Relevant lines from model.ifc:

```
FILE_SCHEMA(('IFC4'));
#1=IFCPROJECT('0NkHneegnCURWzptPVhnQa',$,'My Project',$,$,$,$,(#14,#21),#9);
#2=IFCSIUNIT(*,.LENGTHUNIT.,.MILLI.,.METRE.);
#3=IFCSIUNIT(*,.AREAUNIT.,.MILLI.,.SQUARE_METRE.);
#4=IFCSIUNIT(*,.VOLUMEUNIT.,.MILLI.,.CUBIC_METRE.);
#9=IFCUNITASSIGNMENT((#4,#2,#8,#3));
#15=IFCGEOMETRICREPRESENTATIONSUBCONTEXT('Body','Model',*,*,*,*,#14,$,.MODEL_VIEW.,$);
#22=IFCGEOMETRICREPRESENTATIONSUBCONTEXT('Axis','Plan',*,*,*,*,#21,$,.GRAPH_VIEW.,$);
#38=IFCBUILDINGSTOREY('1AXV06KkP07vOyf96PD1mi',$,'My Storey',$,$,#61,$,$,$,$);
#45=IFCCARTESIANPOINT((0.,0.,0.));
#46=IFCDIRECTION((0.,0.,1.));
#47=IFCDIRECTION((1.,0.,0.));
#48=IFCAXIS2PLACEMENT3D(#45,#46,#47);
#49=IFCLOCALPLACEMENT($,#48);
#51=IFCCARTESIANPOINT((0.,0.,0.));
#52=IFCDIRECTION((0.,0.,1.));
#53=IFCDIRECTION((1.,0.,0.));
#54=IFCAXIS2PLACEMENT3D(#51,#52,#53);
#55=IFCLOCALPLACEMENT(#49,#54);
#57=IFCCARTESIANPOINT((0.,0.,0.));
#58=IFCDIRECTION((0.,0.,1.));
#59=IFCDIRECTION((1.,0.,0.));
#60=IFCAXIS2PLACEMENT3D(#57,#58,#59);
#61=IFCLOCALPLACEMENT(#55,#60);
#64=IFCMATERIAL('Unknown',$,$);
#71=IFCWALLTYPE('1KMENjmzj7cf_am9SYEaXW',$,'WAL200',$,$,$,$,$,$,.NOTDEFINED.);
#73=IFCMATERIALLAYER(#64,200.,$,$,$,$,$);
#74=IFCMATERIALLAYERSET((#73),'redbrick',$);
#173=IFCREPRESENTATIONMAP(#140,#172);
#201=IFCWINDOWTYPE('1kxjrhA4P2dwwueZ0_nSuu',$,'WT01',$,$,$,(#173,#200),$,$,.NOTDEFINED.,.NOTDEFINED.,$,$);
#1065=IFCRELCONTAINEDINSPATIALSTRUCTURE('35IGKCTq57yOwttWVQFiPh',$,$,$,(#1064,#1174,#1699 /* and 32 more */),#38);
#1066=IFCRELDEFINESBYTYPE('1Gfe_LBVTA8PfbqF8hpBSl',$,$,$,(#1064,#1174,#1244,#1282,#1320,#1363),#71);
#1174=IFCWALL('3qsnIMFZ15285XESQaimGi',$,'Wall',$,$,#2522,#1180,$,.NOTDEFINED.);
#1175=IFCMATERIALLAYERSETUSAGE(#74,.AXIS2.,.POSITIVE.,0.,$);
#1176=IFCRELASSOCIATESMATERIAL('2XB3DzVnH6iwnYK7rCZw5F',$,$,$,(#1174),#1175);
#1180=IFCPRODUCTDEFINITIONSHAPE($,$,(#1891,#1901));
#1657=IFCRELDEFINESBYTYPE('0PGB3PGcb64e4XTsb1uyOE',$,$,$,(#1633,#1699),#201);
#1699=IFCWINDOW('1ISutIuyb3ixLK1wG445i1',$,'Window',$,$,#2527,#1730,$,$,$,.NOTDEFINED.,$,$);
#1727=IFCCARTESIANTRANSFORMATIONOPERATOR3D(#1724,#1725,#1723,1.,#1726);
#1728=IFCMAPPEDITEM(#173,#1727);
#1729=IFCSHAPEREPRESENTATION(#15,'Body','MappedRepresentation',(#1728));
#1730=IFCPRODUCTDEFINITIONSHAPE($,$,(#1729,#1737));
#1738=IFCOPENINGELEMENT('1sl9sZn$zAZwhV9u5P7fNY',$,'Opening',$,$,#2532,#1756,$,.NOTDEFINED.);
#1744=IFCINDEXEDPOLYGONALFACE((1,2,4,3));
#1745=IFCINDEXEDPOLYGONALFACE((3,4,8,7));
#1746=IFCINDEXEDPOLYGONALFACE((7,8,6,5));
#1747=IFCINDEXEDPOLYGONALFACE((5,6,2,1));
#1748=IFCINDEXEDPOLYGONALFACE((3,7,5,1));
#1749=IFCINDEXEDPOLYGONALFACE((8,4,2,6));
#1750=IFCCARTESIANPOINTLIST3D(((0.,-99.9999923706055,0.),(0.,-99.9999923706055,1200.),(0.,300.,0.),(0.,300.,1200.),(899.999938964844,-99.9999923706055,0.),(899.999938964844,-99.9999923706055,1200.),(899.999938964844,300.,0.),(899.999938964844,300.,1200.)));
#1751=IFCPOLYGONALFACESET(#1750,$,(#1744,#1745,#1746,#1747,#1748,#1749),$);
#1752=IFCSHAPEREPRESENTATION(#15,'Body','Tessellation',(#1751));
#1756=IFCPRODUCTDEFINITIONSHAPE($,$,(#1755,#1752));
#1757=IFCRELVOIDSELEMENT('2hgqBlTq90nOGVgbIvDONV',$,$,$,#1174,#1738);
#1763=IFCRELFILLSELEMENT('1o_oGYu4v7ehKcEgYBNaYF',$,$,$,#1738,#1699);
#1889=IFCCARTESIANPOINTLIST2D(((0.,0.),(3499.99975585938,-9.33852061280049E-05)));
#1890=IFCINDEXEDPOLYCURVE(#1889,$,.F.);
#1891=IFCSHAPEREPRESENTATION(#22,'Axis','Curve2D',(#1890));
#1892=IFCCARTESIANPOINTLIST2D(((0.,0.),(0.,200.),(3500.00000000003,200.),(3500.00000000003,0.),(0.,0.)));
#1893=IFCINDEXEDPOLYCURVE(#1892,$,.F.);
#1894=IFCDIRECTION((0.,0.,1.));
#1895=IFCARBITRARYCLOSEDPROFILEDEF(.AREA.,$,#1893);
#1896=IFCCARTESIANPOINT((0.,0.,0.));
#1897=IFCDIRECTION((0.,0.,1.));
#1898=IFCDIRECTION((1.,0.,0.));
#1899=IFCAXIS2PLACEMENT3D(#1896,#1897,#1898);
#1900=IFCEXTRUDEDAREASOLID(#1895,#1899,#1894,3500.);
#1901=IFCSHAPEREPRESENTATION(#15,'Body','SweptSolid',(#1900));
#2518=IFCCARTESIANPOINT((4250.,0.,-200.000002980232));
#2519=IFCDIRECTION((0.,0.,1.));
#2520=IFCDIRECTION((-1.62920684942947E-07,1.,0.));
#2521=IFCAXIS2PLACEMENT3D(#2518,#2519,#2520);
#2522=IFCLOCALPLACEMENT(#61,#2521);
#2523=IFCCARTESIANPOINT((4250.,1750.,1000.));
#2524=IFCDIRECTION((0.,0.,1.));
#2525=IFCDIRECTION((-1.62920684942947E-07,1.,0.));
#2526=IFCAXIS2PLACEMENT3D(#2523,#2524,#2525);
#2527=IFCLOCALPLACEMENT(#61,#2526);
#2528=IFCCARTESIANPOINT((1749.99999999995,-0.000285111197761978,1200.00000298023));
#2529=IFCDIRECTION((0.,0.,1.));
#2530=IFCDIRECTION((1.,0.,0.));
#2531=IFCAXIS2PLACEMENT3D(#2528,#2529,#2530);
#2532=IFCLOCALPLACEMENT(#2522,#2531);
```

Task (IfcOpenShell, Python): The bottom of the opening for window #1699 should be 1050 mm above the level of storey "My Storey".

```python
import numpy as np
import ifcopenshell
import ifcopenshell.api.geometry
import ifcopenshell.geom
import ifcopenshell.util.element
import ifcopenshell.util.placement
import ifcopenshell.util.shape
import ifcopenshell.util.unit

model = ifcopenshell.open("model.ifc")
unit_scale = ifcopenshell.util.unit.calculate_unit_scale(model)

window = model.by_id(1699)
opening = window.FillsVoids[0].RelatingOpeningElement
storey = ifcopenshell.util.element.get_container(window, ifc_class="IfcBuildingStorey")
level = ifcopenshell.util.placement.get_local_placement(storey.ObjectPlacement)[2, 3]

# The opening's origin need not be at the sill, so measure its lowest point.
shape = ifcopenshell.geom.create_shape(ifcopenshell.geom.settings(), opening)
bottom = ifcopenshell.util.shape.get_shape_bottom_elevation(shape, shape.geometry) / unit_scale
dz = level + 1.05 / unit_scale - bottom

shift = np.array([0.0, 0.0, dz])
# The window is not placed relative to its opening, so move both.
for product in (opening, window):
    matrix = ifcopenshell.util.placement.get_local_placement(product.ObjectPlacement)
    matrix[:3, 3] += shift
    ifcopenshell.api.geometry.edit_object_placement(model, product=product, matrix=matrix, is_si=False)

print(f"moved by {dz * unit_scale:+.3f} m")

model.write("model_v2.ifc")
```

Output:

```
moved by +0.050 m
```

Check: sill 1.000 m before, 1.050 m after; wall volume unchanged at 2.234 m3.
